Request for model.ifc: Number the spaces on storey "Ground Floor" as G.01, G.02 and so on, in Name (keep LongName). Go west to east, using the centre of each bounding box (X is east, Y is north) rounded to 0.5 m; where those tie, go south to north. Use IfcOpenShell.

First a look at what the model holds.

```python
import ifcopenshell
import ifcopenshell.util.element
import ifcopenshell.util.placement

model = ifcopenshell.open("model.ifc")
print(model.schema)
storey = next(s for s in model.by_type("IfcBuildingStorey") if s.Name == "Ground Floor")
spaces = [e for e in ifcopenshell.util.element.get_decomposition(storey) if e.is_a("IfcSpace")]
for e in sorted(spaces, key=lambda e: e.id()):
    origin = ifcopenshell.util.placement.get_local_placement(e.ObjectPlacement)[:3, 3]
    print(e.id(), e.Name, e.LongName, origin.round(2) + 0.0, sep=" | ")
```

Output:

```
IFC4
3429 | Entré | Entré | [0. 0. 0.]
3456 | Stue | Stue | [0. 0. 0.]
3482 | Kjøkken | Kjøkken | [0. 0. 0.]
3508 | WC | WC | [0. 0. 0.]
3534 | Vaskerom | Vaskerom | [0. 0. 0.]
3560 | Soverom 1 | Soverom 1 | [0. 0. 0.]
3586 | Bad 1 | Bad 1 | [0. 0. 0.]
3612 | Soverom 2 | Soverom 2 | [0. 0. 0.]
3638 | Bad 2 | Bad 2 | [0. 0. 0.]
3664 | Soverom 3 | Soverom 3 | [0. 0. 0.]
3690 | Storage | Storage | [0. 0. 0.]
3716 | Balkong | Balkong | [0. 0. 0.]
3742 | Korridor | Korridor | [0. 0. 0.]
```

```python
import ifcopenshell
import ifcopenshell.geom
import ifcopenshell.util.element
import ifcopenshell.util.shape

model = ifcopenshell.open("model.ifc")
settings = ifcopenshell.geom.settings()
settings.set("use-world-coords", True)


def centre(element):
    shape = ifcopenshell.geom.create_shape(settings, element)
    return ifcopenshell.util.shape.get_bbox_centroid(shape.geometry)


storey = next(s for s in model.by_type("IfcBuildingStorey") if s.Name == "Ground Floor")
spaces = [e for e in ifcopenshell.util.element.get_decomposition(storey) if e.is_a("IfcSpace")]

# Insertion points can sit at a corner or the storey origin, so sort by the geometry (in metres).
centres = {e: centre(e) for e in spaces}
spaces.sort(key=lambda e: (round(centres[e][0] / 0.5), centres[e][1]))

for i, e in enumerate(spaces, start=1):
    number = f"G.{i:02d}"
    e.Name = number
    print(e.id(), number)

model.write("model_v2.ifc")
```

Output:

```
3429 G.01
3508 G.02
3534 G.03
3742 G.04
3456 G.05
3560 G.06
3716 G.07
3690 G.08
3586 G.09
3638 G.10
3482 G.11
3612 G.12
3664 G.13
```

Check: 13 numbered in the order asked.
